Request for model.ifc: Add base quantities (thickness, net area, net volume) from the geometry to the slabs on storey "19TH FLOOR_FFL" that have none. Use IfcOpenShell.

First a look at what the model holds.

```python
import ifcopenshell
import ifcopenshell.util.element
import ifcopenshell.util.unit

model = ifcopenshell.open("model.ifc")
print(model.schema)
for unit_type in ("LENGTHUNIT", "AREAUNIT", "VOLUMEUNIT"):
    print(unit_type, ifcopenshell.util.unit.calculate_unit_scale(model, unit_type))
storey = next(s for s in model.by_type("IfcBuildingStorey") if s.Name == "19TH FLOOR_FFL")
slabs = [e for e in ifcopenshell.util.element.get_decomposition(storey) if e.is_a("IfcSlab")]
for e in sorted(slabs, key=lambda e: e.id()):
    print(e.id(), e.is_a(), e.Name, list(ifcopenshell.util.element.get_psets(e, qtos_only=True)), sep=" | ")
```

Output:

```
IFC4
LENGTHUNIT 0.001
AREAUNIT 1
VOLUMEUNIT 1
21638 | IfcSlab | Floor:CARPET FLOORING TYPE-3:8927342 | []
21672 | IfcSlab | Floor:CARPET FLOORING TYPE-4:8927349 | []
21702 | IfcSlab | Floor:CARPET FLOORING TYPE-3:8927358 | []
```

```python
import ifcopenshell
import ifcopenshell.api.pset
import ifcopenshell.geom
import ifcopenshell.util.element
import ifcopenshell.util.shape
import ifcopenshell.util.unit

model = ifcopenshell.open("model.ifc")
unit_scale = ifcopenshell.util.unit.calculate_unit_scale(model)
area_scale = ifcopenshell.util.unit.calculate_unit_scale(model, "AREAUNIT")
volume_scale = ifcopenshell.util.unit.calculate_unit_scale(model, "VOLUMEUNIT")
settings = ifcopenshell.geom.settings()

storey = next(s for s in model.by_type("IfcBuildingStorey") if s.Name == "19TH FLOOR_FFL")
slabs = [e for e in ifcopenshell.util.element.get_decomposition(storey) if e.is_a("IfcSlab")]

for e in sorted(slabs, key=lambda e: e.id()):
    if ifcopenshell.util.element.get_psets(e, qtos_only=True, should_inherit=False):
        continue
    # Geometry comes back in metres, in the element's own axes.
    shape = ifcopenshell.geom.create_shape(settings, e)
    values = {
        "Width": ifcopenshell.util.shape.get_z(shape.geometry) / unit_scale,
        "NetArea": ifcopenshell.util.shape.get_footprint_area(shape.geometry) / area_scale,
        "NetVolume": ifcopenshell.util.shape.get_volume(shape.geometry) / volume_scale,
    }
    qto = ifcopenshell.api.pset.add_qto(model, product=e, name="Qto_SlabBaseQuantities")
    ifcopenshell.api.pset.edit_qto(model, qto=qto, properties=values)
    print(e.id(), {k: round(v, 3) for k, v in values.items()})

model.write("model-out.ifc")
```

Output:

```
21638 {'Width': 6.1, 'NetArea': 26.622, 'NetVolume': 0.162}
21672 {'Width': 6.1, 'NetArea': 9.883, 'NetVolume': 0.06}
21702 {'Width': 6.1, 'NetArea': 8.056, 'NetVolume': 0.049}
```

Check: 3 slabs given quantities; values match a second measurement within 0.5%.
